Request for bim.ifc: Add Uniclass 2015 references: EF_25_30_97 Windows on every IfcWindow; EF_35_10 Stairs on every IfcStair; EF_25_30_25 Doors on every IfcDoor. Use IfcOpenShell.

First a look at what the model holds.

```python
import ifcopenshell

model = ifcopenshell.open("bim.ifc")
print(model.schema)
print("classifications:", [c.Name for c in model.by_type("IfcClassification")])
for ifc_class in ("IfcDoor", "IfcRoof", "IfcStair", "IfcWall", "IfcWindow"):
    print(ifc_class, len(model.by_type(ifc_class)))
```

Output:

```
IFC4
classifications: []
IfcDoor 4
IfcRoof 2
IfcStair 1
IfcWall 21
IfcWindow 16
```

```python
import ifcopenshell
import ifcopenshell.api.classification

model = ifcopenshell.open("bim.ifc")

system = ifcopenshell.api.classification.add_classification(model, classification="Uniclass 2015")

codes = {
    "IfcWindow": ("EF_25_30_97", "Windows"),
    "IfcStair": ("EF_35_10", "Stairs"),
    "IfcDoor": ("EF_25_30_25", "Doors"),
}
for ifc_class, (code, name) in codes.items():
    products = model.by_type(ifc_class)
    ifcopenshell.api.classification.add_reference(
        model, products=products, classification=system, identification=code, name=name
    )
    print(code, len(products))

model.write("bim-out.ifc")
```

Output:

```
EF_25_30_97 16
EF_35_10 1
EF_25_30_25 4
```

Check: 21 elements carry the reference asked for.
